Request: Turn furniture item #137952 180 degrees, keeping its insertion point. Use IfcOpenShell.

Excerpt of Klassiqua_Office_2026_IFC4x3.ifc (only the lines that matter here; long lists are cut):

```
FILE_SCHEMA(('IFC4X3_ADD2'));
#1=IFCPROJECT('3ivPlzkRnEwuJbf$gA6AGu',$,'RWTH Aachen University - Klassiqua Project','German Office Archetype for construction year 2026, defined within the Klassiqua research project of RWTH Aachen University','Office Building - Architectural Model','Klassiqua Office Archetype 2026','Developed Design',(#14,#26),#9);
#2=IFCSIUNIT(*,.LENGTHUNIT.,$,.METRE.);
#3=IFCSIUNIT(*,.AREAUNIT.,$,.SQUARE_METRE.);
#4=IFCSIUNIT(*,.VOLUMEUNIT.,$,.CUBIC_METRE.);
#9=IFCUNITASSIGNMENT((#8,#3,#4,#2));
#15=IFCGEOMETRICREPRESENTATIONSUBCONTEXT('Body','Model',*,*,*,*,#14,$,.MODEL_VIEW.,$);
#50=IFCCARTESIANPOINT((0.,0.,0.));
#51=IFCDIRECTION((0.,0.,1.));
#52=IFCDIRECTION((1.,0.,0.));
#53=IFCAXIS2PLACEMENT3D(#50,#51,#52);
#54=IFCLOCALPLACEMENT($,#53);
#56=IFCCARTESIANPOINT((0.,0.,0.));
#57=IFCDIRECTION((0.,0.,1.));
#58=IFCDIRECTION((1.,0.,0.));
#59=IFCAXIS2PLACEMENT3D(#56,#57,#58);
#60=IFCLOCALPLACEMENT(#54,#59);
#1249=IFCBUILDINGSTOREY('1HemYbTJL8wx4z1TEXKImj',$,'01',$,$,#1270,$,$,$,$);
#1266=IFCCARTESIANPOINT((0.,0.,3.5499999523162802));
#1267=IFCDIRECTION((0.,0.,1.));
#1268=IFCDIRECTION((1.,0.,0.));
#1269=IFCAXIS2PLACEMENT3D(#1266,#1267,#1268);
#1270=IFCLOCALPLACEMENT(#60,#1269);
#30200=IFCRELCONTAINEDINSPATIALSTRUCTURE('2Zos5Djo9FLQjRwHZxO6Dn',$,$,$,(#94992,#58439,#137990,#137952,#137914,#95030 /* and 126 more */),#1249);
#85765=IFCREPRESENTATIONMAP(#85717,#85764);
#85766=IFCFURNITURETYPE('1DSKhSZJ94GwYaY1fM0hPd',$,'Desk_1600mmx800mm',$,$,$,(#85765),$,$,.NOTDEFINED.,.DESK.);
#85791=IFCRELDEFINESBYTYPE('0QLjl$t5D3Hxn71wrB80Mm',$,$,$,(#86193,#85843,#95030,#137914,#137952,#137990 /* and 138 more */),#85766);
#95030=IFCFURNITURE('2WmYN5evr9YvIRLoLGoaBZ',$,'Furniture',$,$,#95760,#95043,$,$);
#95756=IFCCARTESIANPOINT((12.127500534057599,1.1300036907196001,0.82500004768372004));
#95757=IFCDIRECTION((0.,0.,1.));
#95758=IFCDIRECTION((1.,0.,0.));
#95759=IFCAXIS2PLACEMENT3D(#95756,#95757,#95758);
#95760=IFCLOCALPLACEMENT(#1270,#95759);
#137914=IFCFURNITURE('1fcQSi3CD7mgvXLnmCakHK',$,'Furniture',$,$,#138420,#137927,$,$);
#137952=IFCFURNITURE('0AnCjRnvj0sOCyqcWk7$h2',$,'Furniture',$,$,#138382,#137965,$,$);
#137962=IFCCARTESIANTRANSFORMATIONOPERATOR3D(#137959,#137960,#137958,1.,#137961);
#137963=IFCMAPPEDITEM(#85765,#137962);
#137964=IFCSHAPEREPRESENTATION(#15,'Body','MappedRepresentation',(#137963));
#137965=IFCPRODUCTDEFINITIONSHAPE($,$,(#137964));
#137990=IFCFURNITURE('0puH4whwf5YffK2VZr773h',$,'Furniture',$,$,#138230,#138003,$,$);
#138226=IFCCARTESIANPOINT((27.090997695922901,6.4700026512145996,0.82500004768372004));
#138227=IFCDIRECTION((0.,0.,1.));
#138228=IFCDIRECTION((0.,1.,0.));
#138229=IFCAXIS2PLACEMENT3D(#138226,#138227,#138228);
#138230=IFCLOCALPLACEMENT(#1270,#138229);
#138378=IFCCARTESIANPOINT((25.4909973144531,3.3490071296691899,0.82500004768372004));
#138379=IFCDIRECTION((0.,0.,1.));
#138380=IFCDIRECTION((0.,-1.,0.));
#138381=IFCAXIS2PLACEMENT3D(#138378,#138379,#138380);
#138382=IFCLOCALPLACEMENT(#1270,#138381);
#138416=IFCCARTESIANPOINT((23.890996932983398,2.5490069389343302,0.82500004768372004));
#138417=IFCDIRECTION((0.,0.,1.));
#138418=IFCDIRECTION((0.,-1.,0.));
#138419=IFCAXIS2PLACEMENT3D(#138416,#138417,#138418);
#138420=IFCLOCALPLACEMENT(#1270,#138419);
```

```python
import ifcopenshell
import ifcopenshell.api.geometry
import ifcopenshell.util.placement

model = ifcopenshell.open("Klassiqua_Office_2026_IFC4x3.ifc")

item = model.by_id(137952)
matrix = ifcopenshell.util.placement.get_local_placement(item.ObjectPlacement)
matrix = matrix @ ifcopenshell.util.placement.rotation(180, "Z")
ifcopenshell.api.geometry.edit_object_placement(model, product=item, matrix=matrix, is_si=False)

print(ifcopenshell.util.placement.get_local_placement(item.ObjectPlacement).round(3) + 0.0)

model.write("Klassiqua_Office_2026_IFC4x3_rev.ifc")
```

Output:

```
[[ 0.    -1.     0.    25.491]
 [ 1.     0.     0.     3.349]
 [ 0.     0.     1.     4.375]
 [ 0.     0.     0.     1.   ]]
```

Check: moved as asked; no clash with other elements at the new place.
